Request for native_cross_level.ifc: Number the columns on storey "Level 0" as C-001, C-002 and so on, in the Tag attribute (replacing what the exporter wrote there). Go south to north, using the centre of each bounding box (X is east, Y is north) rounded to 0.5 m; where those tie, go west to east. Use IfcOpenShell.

First a look at what the model holds.

```python
import ifcopenshell
import ifcopenshell.util.element
import ifcopenshell.util.placement

model = ifcopenshell.open("native_cross_level.ifc")
print(model.schema)
storey = next(s for s in model.by_type("IfcBuildingStorey") if s.Name == "Level 0")
columns = [e for e in ifcopenshell.util.element.get_decomposition(storey) if e.is_a("IfcColumn")]
for e in sorted(columns, key=lambda e: e.id()):
    origin = ifcopenshell.util.placement.get_local_placement(e.ObjectPlacement)[:3, 3]
    print(e.id(), e.Tag, e.Name, origin.round(2) + 0.0, sep=" | ")
```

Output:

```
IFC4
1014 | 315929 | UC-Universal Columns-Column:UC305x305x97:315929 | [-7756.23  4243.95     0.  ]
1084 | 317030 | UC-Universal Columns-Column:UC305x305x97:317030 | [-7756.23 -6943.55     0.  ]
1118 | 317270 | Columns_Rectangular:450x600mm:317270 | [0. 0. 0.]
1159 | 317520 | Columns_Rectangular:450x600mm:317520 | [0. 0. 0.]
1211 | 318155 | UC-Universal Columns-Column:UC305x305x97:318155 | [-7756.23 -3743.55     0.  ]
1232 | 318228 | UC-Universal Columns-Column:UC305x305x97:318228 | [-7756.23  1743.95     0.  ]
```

```python
import ifcopenshell
import ifcopenshell.geom
import ifcopenshell.util.element
import ifcopenshell.util.shape

model = ifcopenshell.open("native_cross_level.ifc")
settings = ifcopenshell.geom.settings()
settings.set("use-world-coords", True)


def centre(element):
    shape = ifcopenshell.geom.create_shape(settings, element)
    return ifcopenshell.util.shape.get_bbox_centroid(shape.geometry)


storey = next(s for s in model.by_type("IfcBuildingStorey") if s.Name == "Level 0")
columns = [e for e in ifcopenshell.util.element.get_decomposition(storey) if e.is_a("IfcColumn")]

# Insertion points can sit at a corner or the storey origin, so sort by the geometry (in metres).
centres = {e: centre(e) for e in columns}
columns.sort(key=lambda e: (round(centres[e][1] / 0.5), centres[e][0]))

for i, e in enumerate(columns, start=1):
    number = f"C-0{i:02d}"
    e.Tag = number
    print(e.id(), number)

model.write("native_cross_level_v2.ifc")
```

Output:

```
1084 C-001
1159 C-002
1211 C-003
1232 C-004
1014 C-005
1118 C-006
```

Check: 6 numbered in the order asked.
